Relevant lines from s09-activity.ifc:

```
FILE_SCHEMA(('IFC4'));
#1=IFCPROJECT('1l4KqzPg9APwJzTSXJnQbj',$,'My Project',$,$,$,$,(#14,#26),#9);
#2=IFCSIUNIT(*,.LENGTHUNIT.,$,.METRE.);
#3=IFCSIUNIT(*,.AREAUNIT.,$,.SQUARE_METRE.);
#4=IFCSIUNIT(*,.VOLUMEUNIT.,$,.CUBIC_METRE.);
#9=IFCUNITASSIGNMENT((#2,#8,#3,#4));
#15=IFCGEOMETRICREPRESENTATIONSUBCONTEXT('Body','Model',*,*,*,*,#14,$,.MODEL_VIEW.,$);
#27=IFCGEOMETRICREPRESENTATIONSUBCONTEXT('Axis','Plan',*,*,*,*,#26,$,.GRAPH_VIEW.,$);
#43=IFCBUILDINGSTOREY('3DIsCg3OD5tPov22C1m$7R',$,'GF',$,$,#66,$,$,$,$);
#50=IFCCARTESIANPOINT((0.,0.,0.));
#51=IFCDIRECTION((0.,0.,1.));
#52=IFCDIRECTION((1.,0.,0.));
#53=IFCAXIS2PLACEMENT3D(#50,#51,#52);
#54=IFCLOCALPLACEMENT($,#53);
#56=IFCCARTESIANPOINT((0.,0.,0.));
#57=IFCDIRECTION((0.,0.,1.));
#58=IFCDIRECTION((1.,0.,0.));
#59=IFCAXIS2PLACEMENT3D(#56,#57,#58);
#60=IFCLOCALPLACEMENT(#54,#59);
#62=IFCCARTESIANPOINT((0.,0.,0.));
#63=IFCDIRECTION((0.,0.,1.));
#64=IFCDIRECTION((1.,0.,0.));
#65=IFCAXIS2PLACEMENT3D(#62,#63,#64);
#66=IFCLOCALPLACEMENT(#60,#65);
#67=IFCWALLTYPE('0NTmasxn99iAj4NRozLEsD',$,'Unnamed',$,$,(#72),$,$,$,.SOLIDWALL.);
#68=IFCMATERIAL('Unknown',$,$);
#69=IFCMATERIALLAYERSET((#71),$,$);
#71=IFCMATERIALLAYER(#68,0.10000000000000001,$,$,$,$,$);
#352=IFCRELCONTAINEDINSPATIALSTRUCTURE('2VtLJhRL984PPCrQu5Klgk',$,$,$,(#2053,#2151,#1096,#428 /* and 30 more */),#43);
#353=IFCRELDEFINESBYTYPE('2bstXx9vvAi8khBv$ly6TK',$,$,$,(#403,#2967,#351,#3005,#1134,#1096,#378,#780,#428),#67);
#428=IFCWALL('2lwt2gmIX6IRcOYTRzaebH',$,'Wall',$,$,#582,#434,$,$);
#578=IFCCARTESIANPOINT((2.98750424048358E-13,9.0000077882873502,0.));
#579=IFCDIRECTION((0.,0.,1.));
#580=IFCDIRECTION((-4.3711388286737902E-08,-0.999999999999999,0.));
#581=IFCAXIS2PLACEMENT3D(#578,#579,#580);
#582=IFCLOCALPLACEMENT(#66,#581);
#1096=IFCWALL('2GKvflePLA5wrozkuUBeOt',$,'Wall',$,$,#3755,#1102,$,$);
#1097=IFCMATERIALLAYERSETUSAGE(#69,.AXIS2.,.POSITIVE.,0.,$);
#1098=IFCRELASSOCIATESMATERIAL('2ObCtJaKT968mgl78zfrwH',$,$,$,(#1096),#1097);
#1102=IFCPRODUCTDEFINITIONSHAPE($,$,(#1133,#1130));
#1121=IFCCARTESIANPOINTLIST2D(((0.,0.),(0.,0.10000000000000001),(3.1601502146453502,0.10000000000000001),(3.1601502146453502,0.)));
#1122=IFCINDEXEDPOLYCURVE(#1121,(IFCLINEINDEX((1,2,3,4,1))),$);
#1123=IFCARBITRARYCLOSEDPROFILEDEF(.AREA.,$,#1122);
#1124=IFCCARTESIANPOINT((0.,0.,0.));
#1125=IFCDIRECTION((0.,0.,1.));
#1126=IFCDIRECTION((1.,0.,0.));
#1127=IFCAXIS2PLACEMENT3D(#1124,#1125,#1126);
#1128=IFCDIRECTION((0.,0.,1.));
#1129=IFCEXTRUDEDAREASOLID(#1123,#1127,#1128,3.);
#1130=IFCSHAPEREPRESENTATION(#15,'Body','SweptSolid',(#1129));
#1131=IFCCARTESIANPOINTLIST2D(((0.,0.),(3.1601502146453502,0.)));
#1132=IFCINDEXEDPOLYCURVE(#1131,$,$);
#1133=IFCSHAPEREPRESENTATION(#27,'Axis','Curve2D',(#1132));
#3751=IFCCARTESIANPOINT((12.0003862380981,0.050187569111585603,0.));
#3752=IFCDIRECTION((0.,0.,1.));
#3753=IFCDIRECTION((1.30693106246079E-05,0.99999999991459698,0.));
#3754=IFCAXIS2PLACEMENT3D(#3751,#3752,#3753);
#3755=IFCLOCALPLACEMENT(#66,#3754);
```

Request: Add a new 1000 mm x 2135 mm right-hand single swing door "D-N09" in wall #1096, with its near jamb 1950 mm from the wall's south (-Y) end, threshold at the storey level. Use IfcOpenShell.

```python
import numpy as np
import ifcopenshell
import ifcopenshell.api.feature
import ifcopenshell.api.geometry
import ifcopenshell.api.root
import ifcopenshell.api.spatial
import ifcopenshell.geom
import ifcopenshell.util.element
import ifcopenshell.util.placement
import ifcopenshell.util.representation
import ifcopenshell.util.shape
import ifcopenshell.util.unit

model = ifcopenshell.open("s09-activity.ifc")
unit_scale = ifcopenshell.util.unit.calculate_unit_scale(model)
settings = ifcopenshell.geom.settings()


def volume(element):
    """Net volume in cubic metres, openings subtracted."""
    shape = ifcopenshell.geom.create_shape(settings, element)
    return ifcopenshell.util.shape.get_volume(shape.geometry)


wall = model.by_guid("2GKvflePLA5wrozkuUBeOt")
storey = ifcopenshell.util.element.get_container(wall, ifc_class="IfcBuildingStorey")
context = ifcopenshell.util.representation.get_context(model, "Model", "Body", "MODEL_VIEW")
before = volume(wall)

width, height, from_end, sill = 1, 2.135, 1.95, 0.0  # metres

# The wall runs along its own X axis, and the end named is its -X end.
wall_shape = ifcopenshell.geom.create_shape(settings, wall)
x, y, z = ifcopenshell.util.shape.get_vertices(wall_shape.geometry).T
start = x.min() + from_end
face, thickness = float(y.min()), float(y.max() - y.min())
wall_matrix = ifcopenshell.util.placement.get_local_placement(wall.ObjectPlacement)
level = ifcopenshell.util.placement.get_local_placement(storey.ObjectPlacement)[2, 3]


def in_wall(x, y):
    """Placement at x, y metres in the wall's axes, at sill height."""
    matrix = wall_matrix.copy()
    matrix[:, 3] = wall_matrix @ np.array([x / unit_scale, y / unit_scale, 0.0, 1.0])
    matrix[2, 3] = level + sill / unit_scale
    return matrix


# Opening: a box that overshoots both wall faces by 50 mm.
opening = ifcopenshell.api.root.create_entity(model, ifc_class="IfcOpeningElement", predefined_type="OPENING")
box = ifcopenshell.api.geometry.add_wall_representation(
    model, context=context, length=width, height=height, thickness=thickness + 0.1
)
ifcopenshell.api.geometry.assign_representation(model, product=opening, representation=box)
ifcopenshell.api.geometry.edit_object_placement(model, product=opening, matrix=in_wall(start, face - 0.05), is_si=False)
ifcopenshell.api.feature.add_feature(model, feature=opening, element=wall)

door = ifcopenshell.api.root.create_entity(model, ifc_class="IfcDoor", name="D-N09", predefined_type="DOOR")
door.OverallWidth, door.OverallHeight = width / unit_scale, height / unit_scale
door.OperationType = "SINGLE_SWING_RIGHT"
body = ifcopenshell.api.geometry.add_door_representation(
    model,
    context=context,
    overall_width=door.OverallWidth,
    overall_height=door.OverallHeight,
    operation_type="SINGLE_SWING_RIGHT",
    lining_properties={"LiningDepth": thickness / unit_scale, "ThresholdDepth": thickness / unit_scale},
)
ifcopenshell.api.geometry.assign_representation(model, product=door, representation=body)
ifcopenshell.api.spatial.assign_container(model, products=[door], relating_structure=storey)
ifcopenshell.api.feature.add_filling(model, opening=opening, element=door)

# The lining spans the wall, so the door starts at the wall face.
ifcopenshell.api.geometry.edit_object_placement(model, product=door, matrix=in_wall(start, face), is_si=False)

after = volume(wall)

print(f"wall volume {before:.3f} -> {after:.3f} m3")

model.write("s09-activity_edited.ifc")
```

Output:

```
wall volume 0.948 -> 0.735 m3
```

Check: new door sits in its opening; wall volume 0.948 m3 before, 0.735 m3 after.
